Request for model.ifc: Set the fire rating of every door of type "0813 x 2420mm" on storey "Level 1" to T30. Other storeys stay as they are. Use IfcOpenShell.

First a look at what the model holds.

```python
import ifcopenshell
import ifcopenshell.util.element

model = ifcopenshell.open("model.ifc")
print(model.schema)
storey = next(s for s in model.by_type("IfcBuildingStorey") if s.Name == "Level 1")
doors = [e for e in ifcopenshell.util.element.get_decomposition(storey) if e.is_a("IfcDoor")]
seen = {}
for e in doors:
    element_type = ifcopenshell.util.element.get_type(e)
    key = (element_type.Name if element_type != e and element_type else None, ifcopenshell.util.element.get_pset(e, "Pset_DoorCommon", "FireRating"))
    seen[key] = seen.get(key, 0) + 1
for (name, value), count in sorted(seen.items(), key=str):
    print(count, "x", name, "|", value)
```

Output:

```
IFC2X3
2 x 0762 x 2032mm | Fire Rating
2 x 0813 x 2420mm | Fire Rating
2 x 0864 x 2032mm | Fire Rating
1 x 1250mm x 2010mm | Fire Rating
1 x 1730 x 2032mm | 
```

```python
import ifcopenshell
import ifcopenshell.api.pset
import ifcopenshell.util.element

model = ifcopenshell.open("model.ifc")

storey = next(s for s in model.by_type("IfcBuildingStorey") if s.Name == "Level 1")
doors = [e for e in ifcopenshell.util.element.get_decomposition(storey) if e.is_a("IfcDoor")]

count = 0
for e in doors:
    element_type = ifcopenshell.util.element.get_type(e)
    if element_type in (None, e) or element_type.Name != "0813 x 2420mm":
        continue
    # add_pset returns the element's existing set when there is one.
    pset = ifcopenshell.api.pset.add_pset(model, product=e, name="Pset_DoorCommon")
    ifcopenshell.api.pset.edit_pset(model, pset=pset, properties={"FireRating": "T30"})
    count += 1

print(count, "doors updated")

model.write("model_v2.ifc")
```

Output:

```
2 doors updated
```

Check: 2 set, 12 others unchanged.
